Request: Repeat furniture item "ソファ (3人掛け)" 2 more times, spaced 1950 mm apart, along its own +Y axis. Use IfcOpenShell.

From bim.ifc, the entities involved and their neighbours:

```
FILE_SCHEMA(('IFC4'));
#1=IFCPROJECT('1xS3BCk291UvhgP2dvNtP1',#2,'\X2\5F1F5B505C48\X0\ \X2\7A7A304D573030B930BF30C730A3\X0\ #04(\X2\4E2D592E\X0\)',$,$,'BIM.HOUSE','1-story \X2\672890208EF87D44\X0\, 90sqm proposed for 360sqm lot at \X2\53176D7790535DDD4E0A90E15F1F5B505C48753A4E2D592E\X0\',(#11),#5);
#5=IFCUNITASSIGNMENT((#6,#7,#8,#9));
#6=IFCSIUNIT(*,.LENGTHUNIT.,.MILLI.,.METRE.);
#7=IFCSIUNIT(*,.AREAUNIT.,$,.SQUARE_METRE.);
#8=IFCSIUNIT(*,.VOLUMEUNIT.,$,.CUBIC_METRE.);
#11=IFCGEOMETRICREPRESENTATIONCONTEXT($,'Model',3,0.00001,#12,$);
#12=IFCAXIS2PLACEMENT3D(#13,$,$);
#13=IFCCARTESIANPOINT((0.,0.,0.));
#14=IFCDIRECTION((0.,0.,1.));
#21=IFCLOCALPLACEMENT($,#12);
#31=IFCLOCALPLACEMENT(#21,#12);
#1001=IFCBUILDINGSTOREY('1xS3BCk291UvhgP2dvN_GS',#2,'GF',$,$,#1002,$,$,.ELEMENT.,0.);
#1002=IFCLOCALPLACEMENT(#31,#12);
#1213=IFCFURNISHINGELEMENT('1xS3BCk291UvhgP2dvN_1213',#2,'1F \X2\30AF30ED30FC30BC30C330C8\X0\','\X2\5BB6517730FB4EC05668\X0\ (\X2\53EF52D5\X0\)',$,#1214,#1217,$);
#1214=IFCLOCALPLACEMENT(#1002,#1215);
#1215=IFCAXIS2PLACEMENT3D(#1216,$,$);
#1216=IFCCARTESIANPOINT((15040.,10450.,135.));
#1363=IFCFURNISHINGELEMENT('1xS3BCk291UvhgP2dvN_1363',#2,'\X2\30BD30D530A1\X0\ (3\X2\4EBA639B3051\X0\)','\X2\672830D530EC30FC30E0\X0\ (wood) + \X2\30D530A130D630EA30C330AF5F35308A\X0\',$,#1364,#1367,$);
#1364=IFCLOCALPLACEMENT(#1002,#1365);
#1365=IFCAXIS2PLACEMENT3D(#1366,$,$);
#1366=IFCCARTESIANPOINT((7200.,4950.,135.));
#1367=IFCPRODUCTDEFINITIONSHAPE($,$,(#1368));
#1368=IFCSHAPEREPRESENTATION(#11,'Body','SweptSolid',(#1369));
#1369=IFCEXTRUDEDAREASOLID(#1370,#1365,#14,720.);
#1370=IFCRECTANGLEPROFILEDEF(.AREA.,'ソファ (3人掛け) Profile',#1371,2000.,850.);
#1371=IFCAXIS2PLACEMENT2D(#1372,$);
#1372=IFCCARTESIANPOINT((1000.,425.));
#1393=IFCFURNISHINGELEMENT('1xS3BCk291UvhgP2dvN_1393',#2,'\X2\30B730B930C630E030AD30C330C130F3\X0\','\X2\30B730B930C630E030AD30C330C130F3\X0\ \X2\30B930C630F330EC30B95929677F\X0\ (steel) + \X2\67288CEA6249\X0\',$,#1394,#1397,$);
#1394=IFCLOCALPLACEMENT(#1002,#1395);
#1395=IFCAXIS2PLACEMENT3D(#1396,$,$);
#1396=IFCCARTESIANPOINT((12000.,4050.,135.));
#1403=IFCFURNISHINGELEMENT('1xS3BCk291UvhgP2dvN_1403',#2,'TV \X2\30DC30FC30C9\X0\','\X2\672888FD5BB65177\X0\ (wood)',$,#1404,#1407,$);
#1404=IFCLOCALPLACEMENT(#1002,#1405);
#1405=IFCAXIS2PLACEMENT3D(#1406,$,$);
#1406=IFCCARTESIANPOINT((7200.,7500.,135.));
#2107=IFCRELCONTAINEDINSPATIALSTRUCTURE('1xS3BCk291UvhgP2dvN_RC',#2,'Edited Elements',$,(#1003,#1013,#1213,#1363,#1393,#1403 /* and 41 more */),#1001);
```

```python
import ifcopenshell
import ifcopenshell.api.geometry
import ifcopenshell.api.root
import ifcopenshell.util.element
import ifcopenshell.util.placement

model = ifcopenshell.open("bim.ifc")


def reuse_history(source, copy):
    """copy_class also copies each property set's owner history, people and application; keep the originals."""
    for rel in copy.IsDefinedBy:
        if rel.is_a("IfcRelDefinesByProperties") and (history := rel.RelatingPropertyDefinition.OwnerHistory):
            rel.RelatingPropertyDefinition.OwnerHistory = source.OwnerHistory
            ifcopenshell.util.element.remove_deep2(model, history)


source = model.by_guid("1xS3BCk291UvhgP2dvN_1363")
base = ifcopenshell.util.placement.get_local_placement(source.ObjectPlacement)
step = base[:3, 1] * 1950.0

for i in range(1, 3):
    copy = ifcopenshell.api.root.copy_class(model, product=source)
    copy.Representation = ifcopenshell.util.element.copy_deep(
        model, source.Representation, exclude=["IfcGeometricRepresentationContext", "IfcRepresentationMap"]
    )
    reuse_history(source, copy)
    matrix = base.copy()
    matrix[:3, 3] += i * step
    print("added at", matrix[:3, 3].round(3) + 0.0)
    ifcopenshell.api.geometry.edit_object_placement(model, product=copy, matrix=matrix, is_si=False)

model.write("bim-out.ifc")
```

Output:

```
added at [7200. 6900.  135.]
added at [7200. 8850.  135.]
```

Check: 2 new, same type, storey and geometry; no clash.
